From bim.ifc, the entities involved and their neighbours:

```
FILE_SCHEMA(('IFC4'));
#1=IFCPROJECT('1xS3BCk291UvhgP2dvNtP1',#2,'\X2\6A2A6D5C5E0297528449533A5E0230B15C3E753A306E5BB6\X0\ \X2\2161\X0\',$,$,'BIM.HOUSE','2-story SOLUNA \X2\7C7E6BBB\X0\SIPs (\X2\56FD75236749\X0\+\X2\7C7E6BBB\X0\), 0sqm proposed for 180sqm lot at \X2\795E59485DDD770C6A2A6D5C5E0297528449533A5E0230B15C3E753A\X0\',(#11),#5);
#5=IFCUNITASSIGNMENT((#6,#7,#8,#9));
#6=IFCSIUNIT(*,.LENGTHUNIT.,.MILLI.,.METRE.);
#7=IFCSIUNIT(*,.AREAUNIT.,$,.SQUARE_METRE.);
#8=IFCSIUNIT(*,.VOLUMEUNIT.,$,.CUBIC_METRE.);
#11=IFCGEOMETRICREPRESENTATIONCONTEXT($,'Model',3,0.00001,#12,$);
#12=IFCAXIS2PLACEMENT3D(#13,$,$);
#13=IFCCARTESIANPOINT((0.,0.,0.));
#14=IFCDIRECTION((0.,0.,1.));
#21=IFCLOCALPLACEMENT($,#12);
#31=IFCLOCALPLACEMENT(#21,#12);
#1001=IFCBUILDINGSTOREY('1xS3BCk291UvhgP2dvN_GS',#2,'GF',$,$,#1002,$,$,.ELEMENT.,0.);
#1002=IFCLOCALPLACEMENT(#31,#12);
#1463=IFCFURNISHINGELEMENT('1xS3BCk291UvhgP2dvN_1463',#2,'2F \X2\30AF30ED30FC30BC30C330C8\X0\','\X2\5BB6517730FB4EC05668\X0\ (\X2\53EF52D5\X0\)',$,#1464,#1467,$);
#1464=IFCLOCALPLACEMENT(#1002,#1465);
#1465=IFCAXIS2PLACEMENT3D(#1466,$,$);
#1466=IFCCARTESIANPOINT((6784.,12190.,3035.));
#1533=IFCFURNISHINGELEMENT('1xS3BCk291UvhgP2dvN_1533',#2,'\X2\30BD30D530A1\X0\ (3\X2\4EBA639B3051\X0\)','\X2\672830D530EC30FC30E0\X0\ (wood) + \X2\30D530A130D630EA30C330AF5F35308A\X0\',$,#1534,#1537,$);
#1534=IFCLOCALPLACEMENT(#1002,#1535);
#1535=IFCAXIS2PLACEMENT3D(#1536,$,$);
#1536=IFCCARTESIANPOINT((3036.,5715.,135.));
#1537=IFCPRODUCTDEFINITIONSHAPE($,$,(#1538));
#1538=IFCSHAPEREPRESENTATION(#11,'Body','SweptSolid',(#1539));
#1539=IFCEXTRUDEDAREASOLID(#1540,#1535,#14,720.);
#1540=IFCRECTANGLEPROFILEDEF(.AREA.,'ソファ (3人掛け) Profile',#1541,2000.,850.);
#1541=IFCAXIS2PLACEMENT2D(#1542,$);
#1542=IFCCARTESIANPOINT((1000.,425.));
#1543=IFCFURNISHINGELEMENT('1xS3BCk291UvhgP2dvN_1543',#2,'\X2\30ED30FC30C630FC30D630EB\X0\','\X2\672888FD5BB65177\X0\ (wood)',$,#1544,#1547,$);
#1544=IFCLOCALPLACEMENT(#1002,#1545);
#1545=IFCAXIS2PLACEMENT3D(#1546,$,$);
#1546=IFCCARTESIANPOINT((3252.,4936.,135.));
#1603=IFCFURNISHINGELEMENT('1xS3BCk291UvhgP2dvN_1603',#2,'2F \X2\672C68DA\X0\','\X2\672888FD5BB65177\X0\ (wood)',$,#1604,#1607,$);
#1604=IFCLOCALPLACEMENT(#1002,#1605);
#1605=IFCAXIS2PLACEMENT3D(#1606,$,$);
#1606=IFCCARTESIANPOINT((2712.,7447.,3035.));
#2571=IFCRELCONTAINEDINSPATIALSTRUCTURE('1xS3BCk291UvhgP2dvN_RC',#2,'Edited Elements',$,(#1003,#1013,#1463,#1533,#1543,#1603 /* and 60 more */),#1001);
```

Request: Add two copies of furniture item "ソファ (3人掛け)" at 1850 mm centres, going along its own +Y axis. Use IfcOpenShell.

```python
import ifcopenshell
import ifcopenshell.api.geometry
import ifcopenshell.api.root
import ifcopenshell.util.element
import ifcopenshell.util.placement

model = ifcopenshell.open("bim.ifc")


def reuse_history(source, copy):
    """copy_class also copies each property set's owner history, people and application; keep the originals."""
    for rel in copy.IsDefinedBy:
        if rel.is_a("IfcRelDefinesByProperties") and (history := rel.RelatingPropertyDefinition.OwnerHistory):
            rel.RelatingPropertyDefinition.OwnerHistory = source.OwnerHistory
            ifcopenshell.util.element.remove_deep2(model, history)


source = model.by_id(1533)
base = ifcopenshell.util.placement.get_local_placement(source.ObjectPlacement)
step = base[:3, 1] * 1850.0

for i in range(1, 3):
    copy = ifcopenshell.api.root.copy_class(model, product=source)
    copy.Representation = ifcopenshell.util.element.copy_deep(
        model, source.Representation, exclude=["IfcGeometricRepresentationContext", "IfcRepresentationMap"]
    )
    reuse_history(source, copy)
    matrix = base.copy()
    matrix[:3, 3] += i * step
    print("added at", matrix[:3, 3].round(3) + 0.0)
    ifcopenshell.api.geometry.edit_object_placement(model, product=copy, matrix=matrix, is_si=False)

model.write("bim_rev.ifc")
```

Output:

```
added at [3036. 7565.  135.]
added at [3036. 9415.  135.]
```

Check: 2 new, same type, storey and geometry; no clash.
